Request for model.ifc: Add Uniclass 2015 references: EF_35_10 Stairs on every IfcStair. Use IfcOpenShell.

First a look at what the model holds.

```python
import ifcopenshell

model = ifcopenshell.open("model.ifc")
print(model.schema)
print("classifications:", [c.Name for c in model.by_type("IfcClassification")])
for ifc_class in ("IfcDoor", "IfcRoof", "IfcStair", "IfcWall", "IfcWindow"):
    print(ifc_class, len(model.by_type(ifc_class)))
```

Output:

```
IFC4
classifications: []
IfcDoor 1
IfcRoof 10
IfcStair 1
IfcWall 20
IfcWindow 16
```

```python
import ifcopenshell
import ifcopenshell.api.classification

model = ifcopenshell.open("model.ifc")

system = ifcopenshell.api.classification.add_classification(model, classification="Uniclass 2015")

codes = {
    "IfcStair": ("EF_35_10", "Stairs"),
}
for ifc_class, (code, name) in codes.items():
    products = model.by_type(ifc_class)
    ifcopenshell.api.classification.add_reference(
        model, products=products, classification=system, identification=code, name=name
    )
    print(code, len(products))

model.write("model_rev.ifc")
```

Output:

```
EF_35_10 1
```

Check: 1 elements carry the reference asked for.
